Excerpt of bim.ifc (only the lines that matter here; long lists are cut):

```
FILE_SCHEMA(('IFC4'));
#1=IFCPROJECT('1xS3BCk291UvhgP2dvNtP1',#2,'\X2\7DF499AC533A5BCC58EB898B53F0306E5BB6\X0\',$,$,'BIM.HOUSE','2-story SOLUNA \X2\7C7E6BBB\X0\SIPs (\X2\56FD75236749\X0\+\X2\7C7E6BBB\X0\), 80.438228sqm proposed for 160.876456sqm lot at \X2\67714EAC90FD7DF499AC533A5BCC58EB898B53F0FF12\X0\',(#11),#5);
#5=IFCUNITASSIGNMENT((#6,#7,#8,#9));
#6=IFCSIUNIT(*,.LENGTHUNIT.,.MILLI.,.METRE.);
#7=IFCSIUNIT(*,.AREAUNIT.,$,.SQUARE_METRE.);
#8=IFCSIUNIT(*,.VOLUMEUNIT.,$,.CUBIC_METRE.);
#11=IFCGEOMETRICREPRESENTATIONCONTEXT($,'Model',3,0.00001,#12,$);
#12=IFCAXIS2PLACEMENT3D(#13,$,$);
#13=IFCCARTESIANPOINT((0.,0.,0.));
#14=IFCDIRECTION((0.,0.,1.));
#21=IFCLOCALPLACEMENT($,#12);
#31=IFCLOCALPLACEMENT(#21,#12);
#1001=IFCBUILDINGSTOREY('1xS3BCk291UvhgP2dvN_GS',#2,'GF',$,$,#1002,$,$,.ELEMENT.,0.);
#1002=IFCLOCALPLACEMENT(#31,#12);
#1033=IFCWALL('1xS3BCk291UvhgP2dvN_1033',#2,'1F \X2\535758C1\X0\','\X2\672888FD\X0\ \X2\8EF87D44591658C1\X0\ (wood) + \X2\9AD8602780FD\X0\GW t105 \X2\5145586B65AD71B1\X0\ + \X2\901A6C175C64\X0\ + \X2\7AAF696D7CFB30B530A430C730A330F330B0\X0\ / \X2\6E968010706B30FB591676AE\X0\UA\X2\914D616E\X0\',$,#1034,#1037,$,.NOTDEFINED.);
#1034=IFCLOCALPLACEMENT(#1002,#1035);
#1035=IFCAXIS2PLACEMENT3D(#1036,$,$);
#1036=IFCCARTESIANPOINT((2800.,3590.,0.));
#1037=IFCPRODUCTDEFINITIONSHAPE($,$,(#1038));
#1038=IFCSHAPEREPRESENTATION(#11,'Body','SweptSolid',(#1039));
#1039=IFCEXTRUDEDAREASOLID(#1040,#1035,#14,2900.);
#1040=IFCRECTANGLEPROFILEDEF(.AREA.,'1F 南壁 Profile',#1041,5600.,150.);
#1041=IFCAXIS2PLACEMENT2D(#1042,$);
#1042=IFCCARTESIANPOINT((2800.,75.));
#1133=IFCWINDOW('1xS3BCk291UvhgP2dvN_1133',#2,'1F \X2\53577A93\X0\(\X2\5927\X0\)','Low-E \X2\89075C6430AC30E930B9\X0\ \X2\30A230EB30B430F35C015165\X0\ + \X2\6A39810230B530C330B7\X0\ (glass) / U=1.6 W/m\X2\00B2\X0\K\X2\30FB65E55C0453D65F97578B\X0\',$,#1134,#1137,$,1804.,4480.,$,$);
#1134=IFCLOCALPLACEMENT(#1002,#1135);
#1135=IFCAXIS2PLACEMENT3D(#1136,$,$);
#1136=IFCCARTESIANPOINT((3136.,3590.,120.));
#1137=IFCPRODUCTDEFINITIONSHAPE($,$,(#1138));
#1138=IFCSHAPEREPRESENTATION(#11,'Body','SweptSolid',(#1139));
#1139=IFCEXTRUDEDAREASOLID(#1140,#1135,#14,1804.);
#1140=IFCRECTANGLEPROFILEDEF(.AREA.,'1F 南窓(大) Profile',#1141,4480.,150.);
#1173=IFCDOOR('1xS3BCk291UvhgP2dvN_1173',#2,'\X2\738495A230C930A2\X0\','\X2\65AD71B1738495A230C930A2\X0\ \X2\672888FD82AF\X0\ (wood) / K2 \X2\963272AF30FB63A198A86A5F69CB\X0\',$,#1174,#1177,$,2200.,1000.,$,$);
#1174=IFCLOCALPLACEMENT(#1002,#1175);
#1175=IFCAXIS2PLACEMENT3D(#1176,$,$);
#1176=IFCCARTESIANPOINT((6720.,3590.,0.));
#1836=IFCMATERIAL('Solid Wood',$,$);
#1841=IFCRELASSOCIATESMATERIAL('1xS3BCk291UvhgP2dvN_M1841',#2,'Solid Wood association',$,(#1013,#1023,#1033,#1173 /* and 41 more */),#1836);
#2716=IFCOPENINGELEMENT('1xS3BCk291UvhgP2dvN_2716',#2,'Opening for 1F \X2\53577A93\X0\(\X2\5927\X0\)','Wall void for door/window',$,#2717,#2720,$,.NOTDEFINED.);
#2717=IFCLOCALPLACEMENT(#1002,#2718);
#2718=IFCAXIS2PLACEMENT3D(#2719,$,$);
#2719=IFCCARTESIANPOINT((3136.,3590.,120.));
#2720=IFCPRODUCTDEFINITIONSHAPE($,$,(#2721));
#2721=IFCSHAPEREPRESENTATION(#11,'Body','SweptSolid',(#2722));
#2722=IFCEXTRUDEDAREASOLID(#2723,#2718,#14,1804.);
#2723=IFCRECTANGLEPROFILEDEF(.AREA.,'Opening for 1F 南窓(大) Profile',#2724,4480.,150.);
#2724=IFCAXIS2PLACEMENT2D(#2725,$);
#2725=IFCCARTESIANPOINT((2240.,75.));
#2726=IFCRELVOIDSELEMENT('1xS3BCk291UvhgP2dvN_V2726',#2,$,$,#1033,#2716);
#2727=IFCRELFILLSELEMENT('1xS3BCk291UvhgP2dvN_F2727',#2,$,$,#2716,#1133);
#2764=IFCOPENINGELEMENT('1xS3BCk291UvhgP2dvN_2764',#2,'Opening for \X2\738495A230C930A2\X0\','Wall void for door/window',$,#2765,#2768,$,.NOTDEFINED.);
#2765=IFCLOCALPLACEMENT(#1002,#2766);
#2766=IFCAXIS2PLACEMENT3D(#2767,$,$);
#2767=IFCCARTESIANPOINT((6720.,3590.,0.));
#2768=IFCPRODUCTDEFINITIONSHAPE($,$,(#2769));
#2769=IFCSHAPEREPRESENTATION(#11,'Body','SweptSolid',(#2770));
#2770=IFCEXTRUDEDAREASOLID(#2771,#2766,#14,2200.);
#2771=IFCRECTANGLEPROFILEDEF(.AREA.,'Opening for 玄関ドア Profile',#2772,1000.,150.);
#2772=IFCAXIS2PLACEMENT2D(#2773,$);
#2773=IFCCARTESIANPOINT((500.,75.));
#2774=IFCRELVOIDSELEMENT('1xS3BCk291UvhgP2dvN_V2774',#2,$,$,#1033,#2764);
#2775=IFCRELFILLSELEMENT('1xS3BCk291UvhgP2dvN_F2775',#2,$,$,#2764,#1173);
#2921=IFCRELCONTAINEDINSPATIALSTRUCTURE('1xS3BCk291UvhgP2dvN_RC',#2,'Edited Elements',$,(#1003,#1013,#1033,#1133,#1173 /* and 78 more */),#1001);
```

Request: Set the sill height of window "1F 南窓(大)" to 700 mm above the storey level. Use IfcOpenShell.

```python
import numpy as np
import ifcopenshell
import ifcopenshell.api.geometry
import ifcopenshell.geom
import ifcopenshell.util.element
import ifcopenshell.util.placement
import ifcopenshell.util.shape
import ifcopenshell.util.unit

model = ifcopenshell.open("bim.ifc")
unit_scale = ifcopenshell.util.unit.calculate_unit_scale(model)

window = model.by_guid("1xS3BCk291UvhgP2dvN_1133")
opening = window.FillsVoids[0].RelatingOpeningElement
storey = ifcopenshell.util.element.get_container(window, ifc_class="IfcBuildingStorey")
level = ifcopenshell.util.placement.get_local_placement(storey.ObjectPlacement)[2, 3]

# The opening's origin need not be at the sill, so measure its lowest point.
shape = ifcopenshell.geom.create_shape(ifcopenshell.geom.settings(), opening)
bottom = ifcopenshell.util.shape.get_shape_bottom_elevation(shape, shape.geometry) / unit_scale
dz = level + 0.7 / unit_scale - bottom

shift = np.array([0.0, 0.0, dz])
# The window is not placed relative to its opening, so move both.
for product in (opening, window):
    matrix = ifcopenshell.util.placement.get_local_placement(product.ObjectPlacement)
    matrix[:3, 3] += shift
    ifcopenshell.api.geometry.edit_object_placement(model, product=product, matrix=matrix, is_si=False)

print(f"moved by {dz * unit_scale:+.3f} m")

model.write("bim_updated.ifc")
```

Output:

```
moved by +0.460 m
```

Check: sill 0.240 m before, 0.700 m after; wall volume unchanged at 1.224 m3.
